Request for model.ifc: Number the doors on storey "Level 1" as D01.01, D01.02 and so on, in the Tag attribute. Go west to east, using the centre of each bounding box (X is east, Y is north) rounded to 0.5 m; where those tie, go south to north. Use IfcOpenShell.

First a look at what the model holds.

```python
import ifcopenshell
import ifcopenshell.util.element
import ifcopenshell.util.placement

model = ifcopenshell.open("model.ifc")
print(model.schema)
storey = next(s for s in model.by_type("IfcBuildingStorey") if s.Name == "Level 1")
doors = [e for e in ifcopenshell.util.element.get_decomposition(storey) if e.is_a("IfcDoor")]
for e in sorted(doors, key=lambda e: e.id()):
    origin = ifcopenshell.util.placement.get_local_placement(e.ObjectPlacement)[:3, 3]
    print(e.id(), e.Tag, e.Name, origin.round(2) + 0.0, sep=" | ")
```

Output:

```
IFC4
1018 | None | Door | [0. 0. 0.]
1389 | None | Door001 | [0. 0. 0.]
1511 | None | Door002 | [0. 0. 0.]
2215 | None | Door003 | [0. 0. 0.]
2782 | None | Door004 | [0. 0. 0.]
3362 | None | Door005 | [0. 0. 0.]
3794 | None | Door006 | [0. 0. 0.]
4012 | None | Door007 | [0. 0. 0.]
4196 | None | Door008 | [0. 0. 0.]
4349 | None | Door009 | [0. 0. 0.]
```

```python
import ifcopenshell
import ifcopenshell.geom
import ifcopenshell.util.element
import ifcopenshell.util.shape

model = ifcopenshell.open("model.ifc")
settings = ifcopenshell.geom.settings()
settings.set("use-world-coords", True)


def centre(element):
    shape = ifcopenshell.geom.create_shape(settings, element)
    return ifcopenshell.util.shape.get_bbox_centroid(shape.geometry)


storey = next(s for s in model.by_type("IfcBuildingStorey") if s.Name == "Level 1")
doors = [e for e in ifcopenshell.util.element.get_decomposition(storey) if e.is_a("IfcDoor")]

# Insertion points can sit at a corner or the storey origin, so sort by the geometry (in metres).
centres = {e: centre(e) for e in doors}
doors.sort(key=lambda e: (round(centres[e][0] / 0.5), centres[e][1]))

for i, e in enumerate(doors, start=1):
    number = f"D01.{i:02d}"
    e.Tag = number
    print(e.id(), number)

model.write("model_v2.ifc")
```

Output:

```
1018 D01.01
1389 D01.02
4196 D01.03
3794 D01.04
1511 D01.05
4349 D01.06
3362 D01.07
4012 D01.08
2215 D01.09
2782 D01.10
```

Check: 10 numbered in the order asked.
